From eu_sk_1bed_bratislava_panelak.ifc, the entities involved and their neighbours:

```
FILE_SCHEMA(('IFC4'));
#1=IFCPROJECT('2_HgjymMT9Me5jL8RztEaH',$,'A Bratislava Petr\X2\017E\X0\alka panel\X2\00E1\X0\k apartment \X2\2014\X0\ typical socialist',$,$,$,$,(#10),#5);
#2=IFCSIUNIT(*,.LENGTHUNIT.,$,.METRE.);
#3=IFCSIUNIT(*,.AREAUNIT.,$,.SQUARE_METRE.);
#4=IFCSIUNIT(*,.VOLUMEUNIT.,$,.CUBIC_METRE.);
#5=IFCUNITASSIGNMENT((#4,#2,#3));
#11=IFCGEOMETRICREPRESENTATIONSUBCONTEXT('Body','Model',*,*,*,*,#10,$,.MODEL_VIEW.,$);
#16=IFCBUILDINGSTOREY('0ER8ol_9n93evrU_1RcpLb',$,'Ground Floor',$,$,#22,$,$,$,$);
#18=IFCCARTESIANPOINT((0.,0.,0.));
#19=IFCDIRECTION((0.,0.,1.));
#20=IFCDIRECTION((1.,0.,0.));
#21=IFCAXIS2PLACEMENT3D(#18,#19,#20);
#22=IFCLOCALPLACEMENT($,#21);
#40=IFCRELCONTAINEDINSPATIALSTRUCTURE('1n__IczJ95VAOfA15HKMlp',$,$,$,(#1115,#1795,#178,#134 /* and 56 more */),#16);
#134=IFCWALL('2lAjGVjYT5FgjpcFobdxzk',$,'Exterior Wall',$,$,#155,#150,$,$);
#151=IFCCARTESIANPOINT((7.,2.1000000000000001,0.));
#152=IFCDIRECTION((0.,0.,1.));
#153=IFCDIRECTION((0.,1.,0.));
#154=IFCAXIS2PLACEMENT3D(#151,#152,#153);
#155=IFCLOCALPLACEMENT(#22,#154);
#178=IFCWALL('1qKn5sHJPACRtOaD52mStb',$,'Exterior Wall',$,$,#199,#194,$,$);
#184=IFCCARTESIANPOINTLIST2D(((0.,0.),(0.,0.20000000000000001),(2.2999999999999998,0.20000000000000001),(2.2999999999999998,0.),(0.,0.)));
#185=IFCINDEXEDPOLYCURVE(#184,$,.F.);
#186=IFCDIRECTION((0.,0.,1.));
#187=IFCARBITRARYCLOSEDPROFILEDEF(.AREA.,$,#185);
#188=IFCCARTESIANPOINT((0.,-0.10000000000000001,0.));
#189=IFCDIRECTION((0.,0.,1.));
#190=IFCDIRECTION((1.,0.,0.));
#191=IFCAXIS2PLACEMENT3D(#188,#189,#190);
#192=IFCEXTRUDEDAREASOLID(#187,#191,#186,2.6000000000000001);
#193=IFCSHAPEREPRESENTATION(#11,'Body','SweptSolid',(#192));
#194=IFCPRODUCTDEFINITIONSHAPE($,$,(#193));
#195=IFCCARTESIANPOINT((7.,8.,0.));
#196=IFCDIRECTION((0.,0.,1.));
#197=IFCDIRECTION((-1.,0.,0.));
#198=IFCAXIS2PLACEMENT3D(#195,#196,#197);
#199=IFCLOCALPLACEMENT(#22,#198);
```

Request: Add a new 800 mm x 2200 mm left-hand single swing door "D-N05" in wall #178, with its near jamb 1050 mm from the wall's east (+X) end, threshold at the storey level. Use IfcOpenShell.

```python
import numpy as np
import ifcopenshell
import ifcopenshell.api.feature
import ifcopenshell.api.geometry
import ifcopenshell.api.root
import ifcopenshell.api.spatial
import ifcopenshell.geom
import ifcopenshell.util.element
import ifcopenshell.util.placement
import ifcopenshell.util.representation
import ifcopenshell.util.shape
import ifcopenshell.util.unit

model = ifcopenshell.open("eu_sk_1bed_bratislava_panelak.ifc")
unit_scale = ifcopenshell.util.unit.calculate_unit_scale(model)
settings = ifcopenshell.geom.settings()


def volume(element):
    """Net volume in cubic metres, openings subtracted."""
    shape = ifcopenshell.geom.create_shape(settings, element)
    return ifcopenshell.util.shape.get_volume(shape.geometry)


wall = model.by_guid("1qKn5sHJPACRtOaD52mStb")
storey = ifcopenshell.util.element.get_container(wall, ifc_class="IfcBuildingStorey")
context = ifcopenshell.util.representation.get_context(model, "Model", "Body", "MODEL_VIEW")
before = volume(wall)

width, height, from_end, sill = 0.8, 2.2, 1.05, 0.0  # metres

# The wall runs along its own X axis, and the end named is its -X end.
wall_shape = ifcopenshell.geom.create_shape(settings, wall)
x, y, z = ifcopenshell.util.shape.get_vertices(wall_shape.geometry).T
start = x.min() + from_end
face, thickness = float(y.min()), float(y.max() - y.min())
wall_matrix = ifcopenshell.util.placement.get_local_placement(wall.ObjectPlacement)
level = ifcopenshell.util.placement.get_local_placement(storey.ObjectPlacement)[2, 3]


def in_wall(x, y):
    """Placement at x, y metres in the wall's axes, at sill height."""
    matrix = wall_matrix.copy()
    matrix[:, 3] = wall_matrix @ np.array([x / unit_scale, y / unit_scale, 0.0, 1.0])
    matrix[2, 3] = level + sill / unit_scale
    return matrix


# Opening: a box that overshoots both wall faces by 50 mm.
opening = ifcopenshell.api.root.create_entity(model, ifc_class="IfcOpeningElement", predefined_type="OPENING")
box = ifcopenshell.api.geometry.add_wall_representation(
    model, context=context, length=width, height=height, thickness=thickness + 0.1
)
ifcopenshell.api.geometry.assign_representation(model, product=opening, representation=box)
ifcopenshell.api.geometry.edit_object_placement(model, product=opening, matrix=in_wall(start, face - 0.05), is_si=False)
ifcopenshell.api.feature.add_feature(model, feature=opening, element=wall)

door = ifcopenshell.api.root.create_entity(model, ifc_class="IfcDoor", name="D-N05", predefined_type="DOOR")
door.OverallWidth, door.OverallHeight = width / unit_scale, height / unit_scale
door.OperationType = "SINGLE_SWING_LEFT"
body = ifcopenshell.api.geometry.add_door_representation(
    model,
    context=context,
    overall_width=door.OverallWidth,
    overall_height=door.OverallHeight,
    operation_type="SINGLE_SWING_LEFT",
    lining_properties={"LiningDepth": thickness / unit_scale, "ThresholdDepth": thickness / unit_scale},
)
ifcopenshell.api.geometry.assign_representation(model, product=door, representation=body)
ifcopenshell.api.spatial.assign_container(model, products=[door], relating_structure=storey)
ifcopenshell.api.feature.add_filling(model, opening=opening, element=door)

# The lining spans the wall, so the door starts at the wall face.
ifcopenshell.api.geometry.edit_object_placement(model, product=door, matrix=in_wall(start, face), is_si=False)

after = volume(wall)

print(f"wall volume {before:.3f} -> {after:.3f} m3")

model.write("eu_sk_1bed_bratislava_panelak_v2.ifc")
```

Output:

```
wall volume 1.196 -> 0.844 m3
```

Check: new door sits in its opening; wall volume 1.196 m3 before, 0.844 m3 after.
